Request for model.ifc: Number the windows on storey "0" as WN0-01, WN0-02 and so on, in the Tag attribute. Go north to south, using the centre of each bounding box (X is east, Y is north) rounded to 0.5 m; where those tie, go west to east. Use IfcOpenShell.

First a look at what the model holds.

```python
import ifcopenshell
import ifcopenshell.util.element
import ifcopenshell.util.placement

model = ifcopenshell.open("model.ifc")
print(model.schema)
storey = next(s for s in model.by_type("IfcBuildingStorey") if s.Name == "0")
windows = [e for e in ifcopenshell.util.element.get_decomposition(storey) if e.is_a("IfcWindow")]
for e in sorted(windows, key=lambda e: e.id()):
    origin = ifcopenshell.util.placement.get_local_placement(e.ObjectPlacement)[:3, 3]
    print(e.id(), e.Tag, e.Name, origin.round(2) + 0.0, sep=" | ")
```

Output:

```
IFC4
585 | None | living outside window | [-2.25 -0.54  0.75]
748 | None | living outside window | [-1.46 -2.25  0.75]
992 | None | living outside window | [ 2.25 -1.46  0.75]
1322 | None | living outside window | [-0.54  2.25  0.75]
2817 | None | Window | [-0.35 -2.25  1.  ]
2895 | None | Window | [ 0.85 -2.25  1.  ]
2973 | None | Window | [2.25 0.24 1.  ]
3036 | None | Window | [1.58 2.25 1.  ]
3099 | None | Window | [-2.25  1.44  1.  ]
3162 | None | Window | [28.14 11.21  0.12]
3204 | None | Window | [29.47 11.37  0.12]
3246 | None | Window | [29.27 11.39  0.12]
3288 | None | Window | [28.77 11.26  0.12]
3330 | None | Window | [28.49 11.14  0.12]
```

```python
import ifcopenshell
import ifcopenshell.geom
import ifcopenshell.util.element
import ifcopenshell.util.shape

model = ifcopenshell.open("model.ifc")
settings = ifcopenshell.geom.settings()
settings.set("use-world-coords", True)


def centre(element):
    shape = ifcopenshell.geom.create_shape(settings, element)
    return ifcopenshell.util.shape.get_bbox_centroid(shape.geometry)


storey = next(s for s in model.by_type("IfcBuildingStorey") if s.Name == "0")
windows = [e for e in ifcopenshell.util.element.get_decomposition(storey) if e.is_a("IfcWindow")]

# Insertion points can sit at a corner or the storey origin, so sort by the geometry (in metres).
centres = {e: centre(e) for e in windows}
windows.sort(key=lambda e: (-round(centres[e][1] / 0.5), centres[e][0]))

for i, e in enumerate(windows, start=1):
    number = f"WN0-{i:02d}"
    e.Tag = number
    print(e.id(), number)

model.write("model_edited.ifc")
```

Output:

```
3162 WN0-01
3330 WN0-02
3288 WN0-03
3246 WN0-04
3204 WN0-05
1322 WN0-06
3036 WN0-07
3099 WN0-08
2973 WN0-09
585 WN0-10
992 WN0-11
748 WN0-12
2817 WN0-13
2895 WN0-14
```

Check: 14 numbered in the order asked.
